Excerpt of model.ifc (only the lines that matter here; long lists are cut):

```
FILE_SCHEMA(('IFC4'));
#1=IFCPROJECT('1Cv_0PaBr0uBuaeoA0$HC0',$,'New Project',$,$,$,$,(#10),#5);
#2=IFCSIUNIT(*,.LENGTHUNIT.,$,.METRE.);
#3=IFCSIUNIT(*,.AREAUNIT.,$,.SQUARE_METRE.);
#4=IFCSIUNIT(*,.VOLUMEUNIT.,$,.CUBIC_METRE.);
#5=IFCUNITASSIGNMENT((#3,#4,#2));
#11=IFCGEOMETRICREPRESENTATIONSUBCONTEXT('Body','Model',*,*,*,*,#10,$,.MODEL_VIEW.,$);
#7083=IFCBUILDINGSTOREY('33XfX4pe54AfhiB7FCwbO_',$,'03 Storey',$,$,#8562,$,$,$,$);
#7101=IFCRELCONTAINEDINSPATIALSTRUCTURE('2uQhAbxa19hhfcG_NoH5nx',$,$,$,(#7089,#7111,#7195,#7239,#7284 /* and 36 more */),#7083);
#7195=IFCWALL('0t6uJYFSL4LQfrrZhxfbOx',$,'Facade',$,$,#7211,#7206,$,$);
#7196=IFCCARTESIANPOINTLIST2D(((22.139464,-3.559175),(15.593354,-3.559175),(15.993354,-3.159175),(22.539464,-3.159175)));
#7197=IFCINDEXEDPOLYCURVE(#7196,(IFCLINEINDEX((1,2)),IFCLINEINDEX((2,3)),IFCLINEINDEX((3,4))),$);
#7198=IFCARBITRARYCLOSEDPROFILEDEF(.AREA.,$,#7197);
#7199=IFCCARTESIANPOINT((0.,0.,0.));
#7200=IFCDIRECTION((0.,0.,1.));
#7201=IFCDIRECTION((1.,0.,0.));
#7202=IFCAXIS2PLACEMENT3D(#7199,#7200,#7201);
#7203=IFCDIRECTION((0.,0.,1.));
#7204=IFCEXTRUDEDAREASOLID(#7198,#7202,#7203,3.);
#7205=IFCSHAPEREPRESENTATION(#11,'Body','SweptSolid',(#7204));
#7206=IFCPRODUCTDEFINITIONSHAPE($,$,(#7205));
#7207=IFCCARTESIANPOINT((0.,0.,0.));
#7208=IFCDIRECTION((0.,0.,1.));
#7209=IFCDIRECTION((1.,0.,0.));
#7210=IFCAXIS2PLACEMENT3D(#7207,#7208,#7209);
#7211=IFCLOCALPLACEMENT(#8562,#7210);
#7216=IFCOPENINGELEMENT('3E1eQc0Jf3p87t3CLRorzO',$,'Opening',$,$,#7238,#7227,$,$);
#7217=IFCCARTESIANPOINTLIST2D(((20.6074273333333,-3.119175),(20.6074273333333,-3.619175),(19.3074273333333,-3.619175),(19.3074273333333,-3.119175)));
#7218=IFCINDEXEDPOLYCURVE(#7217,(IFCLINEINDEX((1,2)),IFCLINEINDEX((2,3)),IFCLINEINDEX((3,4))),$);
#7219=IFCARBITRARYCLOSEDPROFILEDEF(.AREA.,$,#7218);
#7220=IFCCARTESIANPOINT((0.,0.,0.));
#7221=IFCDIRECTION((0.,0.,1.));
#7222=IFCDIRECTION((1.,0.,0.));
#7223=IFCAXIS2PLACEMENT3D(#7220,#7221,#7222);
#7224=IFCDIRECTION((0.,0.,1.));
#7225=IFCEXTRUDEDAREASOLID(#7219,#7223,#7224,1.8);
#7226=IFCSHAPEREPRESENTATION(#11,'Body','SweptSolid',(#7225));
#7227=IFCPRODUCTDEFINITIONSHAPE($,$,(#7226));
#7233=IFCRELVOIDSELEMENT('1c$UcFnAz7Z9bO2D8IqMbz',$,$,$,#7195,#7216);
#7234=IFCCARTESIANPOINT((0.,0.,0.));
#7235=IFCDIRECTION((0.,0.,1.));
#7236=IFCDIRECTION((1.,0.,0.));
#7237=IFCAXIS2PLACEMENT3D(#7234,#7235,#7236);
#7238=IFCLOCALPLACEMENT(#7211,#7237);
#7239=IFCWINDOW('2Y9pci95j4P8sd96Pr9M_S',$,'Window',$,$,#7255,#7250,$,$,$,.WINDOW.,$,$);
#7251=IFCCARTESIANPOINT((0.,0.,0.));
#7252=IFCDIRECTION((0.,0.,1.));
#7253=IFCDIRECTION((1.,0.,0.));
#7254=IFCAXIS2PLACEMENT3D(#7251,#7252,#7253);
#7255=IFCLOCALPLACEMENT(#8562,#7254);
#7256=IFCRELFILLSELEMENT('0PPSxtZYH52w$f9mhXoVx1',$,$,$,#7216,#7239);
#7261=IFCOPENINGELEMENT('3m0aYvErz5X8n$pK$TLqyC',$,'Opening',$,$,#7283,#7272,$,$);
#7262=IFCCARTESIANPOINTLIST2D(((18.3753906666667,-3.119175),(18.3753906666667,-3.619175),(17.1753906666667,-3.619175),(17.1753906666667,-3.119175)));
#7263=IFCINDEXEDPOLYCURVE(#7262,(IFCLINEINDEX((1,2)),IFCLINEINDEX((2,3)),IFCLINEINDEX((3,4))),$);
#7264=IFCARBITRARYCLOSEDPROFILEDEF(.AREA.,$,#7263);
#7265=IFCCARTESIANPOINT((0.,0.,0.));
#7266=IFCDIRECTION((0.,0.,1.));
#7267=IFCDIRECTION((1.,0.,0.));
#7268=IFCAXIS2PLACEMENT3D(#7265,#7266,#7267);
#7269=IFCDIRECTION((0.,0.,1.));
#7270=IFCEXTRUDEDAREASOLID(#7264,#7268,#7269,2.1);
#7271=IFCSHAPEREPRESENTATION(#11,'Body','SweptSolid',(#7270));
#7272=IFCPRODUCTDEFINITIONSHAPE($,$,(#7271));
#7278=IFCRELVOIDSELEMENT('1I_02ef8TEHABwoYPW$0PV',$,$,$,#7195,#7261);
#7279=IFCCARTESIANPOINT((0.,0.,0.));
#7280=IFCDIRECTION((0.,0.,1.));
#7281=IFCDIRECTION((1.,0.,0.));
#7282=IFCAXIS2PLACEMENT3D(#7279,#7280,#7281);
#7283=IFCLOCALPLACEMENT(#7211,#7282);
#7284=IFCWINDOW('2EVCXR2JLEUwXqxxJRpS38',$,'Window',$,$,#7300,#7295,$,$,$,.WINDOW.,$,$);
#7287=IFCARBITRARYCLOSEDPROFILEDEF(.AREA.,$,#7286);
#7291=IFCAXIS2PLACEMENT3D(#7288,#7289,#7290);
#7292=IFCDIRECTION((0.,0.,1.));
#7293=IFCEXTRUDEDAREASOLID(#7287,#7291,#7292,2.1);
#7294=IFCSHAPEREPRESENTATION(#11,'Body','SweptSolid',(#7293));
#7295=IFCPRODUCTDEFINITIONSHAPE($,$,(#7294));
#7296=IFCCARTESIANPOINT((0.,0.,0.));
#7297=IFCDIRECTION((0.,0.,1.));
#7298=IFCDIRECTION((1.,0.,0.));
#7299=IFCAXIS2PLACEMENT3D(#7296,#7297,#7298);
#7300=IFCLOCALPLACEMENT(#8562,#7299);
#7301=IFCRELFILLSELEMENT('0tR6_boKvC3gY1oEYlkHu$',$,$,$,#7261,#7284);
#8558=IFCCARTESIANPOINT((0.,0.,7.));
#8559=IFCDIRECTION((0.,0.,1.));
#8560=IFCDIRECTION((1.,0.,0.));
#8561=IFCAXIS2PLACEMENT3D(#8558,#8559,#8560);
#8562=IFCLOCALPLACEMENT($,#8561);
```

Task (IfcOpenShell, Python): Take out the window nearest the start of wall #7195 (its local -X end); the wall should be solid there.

```python
import ifcopenshell
import ifcopenshell.api.feature
import ifcopenshell.api.root
import ifcopenshell.geom
import ifcopenshell.util.shape

model = ifcopenshell.open("model.ifc")
settings = ifcopenshell.geom.settings()


def volume(element):
    """Net volume in cubic metres, openings subtracted."""
    shape = ifcopenshell.geom.create_shape(settings, element)
    return ifcopenshell.util.shape.get_volume(shape.geometry)


window = model.by_guid("2EVCXR2JLEUwXqxxJRpS38")
opening = window.FillsVoids[0].RelatingOpeningElement
wall = opening.VoidsElements[0].RelatingBuildingElement
before = volume(wall)

ifcopenshell.api.root.remove_product(model, product=window)
ifcopenshell.api.feature.remove_feature(model, feature=opening)

after = volume(wall)

print(f"wall volume {before:.3f} -> {after:.3f} m3")

model.write("model_updated.ifc")
```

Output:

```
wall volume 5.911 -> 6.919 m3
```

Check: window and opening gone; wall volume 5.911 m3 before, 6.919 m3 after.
